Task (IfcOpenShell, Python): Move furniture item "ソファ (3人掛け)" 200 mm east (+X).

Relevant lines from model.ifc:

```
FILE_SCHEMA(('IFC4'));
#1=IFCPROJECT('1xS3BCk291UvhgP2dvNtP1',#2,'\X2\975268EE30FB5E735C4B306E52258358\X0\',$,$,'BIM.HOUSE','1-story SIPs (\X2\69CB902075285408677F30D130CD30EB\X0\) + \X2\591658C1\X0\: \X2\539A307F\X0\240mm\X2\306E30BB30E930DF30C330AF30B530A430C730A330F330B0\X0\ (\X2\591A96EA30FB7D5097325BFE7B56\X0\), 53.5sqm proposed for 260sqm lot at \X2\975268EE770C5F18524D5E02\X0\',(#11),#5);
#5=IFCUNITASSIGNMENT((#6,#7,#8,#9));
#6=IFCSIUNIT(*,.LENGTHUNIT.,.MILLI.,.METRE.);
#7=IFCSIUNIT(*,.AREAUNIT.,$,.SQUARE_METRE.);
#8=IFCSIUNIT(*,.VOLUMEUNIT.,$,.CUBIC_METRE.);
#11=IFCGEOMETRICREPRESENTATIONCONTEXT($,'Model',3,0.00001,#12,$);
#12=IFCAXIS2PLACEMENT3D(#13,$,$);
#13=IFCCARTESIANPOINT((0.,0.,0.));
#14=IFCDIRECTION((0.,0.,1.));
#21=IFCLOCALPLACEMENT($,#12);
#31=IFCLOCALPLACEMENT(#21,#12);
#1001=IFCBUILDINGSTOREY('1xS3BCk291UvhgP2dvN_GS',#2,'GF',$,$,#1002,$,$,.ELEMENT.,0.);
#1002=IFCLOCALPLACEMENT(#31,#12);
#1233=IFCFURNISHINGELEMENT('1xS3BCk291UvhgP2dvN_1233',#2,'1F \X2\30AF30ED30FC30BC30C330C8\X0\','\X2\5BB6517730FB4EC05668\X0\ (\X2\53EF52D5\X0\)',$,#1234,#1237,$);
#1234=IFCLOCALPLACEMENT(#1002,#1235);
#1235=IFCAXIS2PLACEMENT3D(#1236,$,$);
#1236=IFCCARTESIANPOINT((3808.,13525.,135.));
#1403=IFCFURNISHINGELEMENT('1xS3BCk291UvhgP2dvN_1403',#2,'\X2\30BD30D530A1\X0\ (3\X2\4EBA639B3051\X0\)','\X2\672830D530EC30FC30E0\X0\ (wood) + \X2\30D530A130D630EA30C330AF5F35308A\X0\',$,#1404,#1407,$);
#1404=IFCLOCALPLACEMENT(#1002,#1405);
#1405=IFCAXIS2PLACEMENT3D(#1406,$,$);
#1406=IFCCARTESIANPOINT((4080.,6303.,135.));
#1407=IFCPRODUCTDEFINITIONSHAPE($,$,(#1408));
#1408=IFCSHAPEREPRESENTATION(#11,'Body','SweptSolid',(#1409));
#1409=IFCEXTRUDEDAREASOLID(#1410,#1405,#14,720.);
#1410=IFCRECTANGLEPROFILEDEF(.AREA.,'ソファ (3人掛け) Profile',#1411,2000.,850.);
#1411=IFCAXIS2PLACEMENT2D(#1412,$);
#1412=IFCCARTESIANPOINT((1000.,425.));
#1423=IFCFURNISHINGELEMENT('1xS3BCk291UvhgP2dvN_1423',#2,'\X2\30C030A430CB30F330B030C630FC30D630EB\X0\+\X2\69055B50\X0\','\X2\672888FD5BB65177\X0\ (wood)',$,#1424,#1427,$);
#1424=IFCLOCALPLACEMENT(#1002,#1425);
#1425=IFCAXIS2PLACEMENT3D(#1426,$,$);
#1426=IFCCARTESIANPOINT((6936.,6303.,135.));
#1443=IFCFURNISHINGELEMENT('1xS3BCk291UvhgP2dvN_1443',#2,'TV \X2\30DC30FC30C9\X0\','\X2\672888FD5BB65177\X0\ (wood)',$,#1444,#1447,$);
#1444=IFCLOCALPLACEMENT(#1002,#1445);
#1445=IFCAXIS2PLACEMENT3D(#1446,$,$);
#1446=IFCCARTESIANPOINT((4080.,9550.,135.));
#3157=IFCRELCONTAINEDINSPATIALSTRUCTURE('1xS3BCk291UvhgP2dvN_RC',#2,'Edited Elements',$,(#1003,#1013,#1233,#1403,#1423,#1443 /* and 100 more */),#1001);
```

```python
import ifcopenshell
import ifcopenshell.api.geometry
import ifcopenshell.util.placement
import ifcopenshell.util.unit

model = ifcopenshell.open("model.ifc")
unit_scale = ifcopenshell.util.unit.calculate_unit_scale(model)

item = model.by_guid("1xS3BCk291UvhgP2dvN_1403")
matrix = ifcopenshell.util.placement.get_local_placement(item.ObjectPlacement)
matrix[0, 3] += 0.2 / unit_scale
ifcopenshell.api.geometry.edit_object_placement(model, product=item, matrix=matrix, is_si=False)

print(ifcopenshell.util.placement.get_local_placement(item.ObjectPlacement).round(3) + 0.0)

model.write("model_rev.ifc")
```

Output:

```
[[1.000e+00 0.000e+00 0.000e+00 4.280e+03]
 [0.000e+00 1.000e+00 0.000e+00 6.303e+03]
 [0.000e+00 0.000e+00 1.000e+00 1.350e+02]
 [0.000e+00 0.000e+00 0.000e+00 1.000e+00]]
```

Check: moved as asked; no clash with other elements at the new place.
